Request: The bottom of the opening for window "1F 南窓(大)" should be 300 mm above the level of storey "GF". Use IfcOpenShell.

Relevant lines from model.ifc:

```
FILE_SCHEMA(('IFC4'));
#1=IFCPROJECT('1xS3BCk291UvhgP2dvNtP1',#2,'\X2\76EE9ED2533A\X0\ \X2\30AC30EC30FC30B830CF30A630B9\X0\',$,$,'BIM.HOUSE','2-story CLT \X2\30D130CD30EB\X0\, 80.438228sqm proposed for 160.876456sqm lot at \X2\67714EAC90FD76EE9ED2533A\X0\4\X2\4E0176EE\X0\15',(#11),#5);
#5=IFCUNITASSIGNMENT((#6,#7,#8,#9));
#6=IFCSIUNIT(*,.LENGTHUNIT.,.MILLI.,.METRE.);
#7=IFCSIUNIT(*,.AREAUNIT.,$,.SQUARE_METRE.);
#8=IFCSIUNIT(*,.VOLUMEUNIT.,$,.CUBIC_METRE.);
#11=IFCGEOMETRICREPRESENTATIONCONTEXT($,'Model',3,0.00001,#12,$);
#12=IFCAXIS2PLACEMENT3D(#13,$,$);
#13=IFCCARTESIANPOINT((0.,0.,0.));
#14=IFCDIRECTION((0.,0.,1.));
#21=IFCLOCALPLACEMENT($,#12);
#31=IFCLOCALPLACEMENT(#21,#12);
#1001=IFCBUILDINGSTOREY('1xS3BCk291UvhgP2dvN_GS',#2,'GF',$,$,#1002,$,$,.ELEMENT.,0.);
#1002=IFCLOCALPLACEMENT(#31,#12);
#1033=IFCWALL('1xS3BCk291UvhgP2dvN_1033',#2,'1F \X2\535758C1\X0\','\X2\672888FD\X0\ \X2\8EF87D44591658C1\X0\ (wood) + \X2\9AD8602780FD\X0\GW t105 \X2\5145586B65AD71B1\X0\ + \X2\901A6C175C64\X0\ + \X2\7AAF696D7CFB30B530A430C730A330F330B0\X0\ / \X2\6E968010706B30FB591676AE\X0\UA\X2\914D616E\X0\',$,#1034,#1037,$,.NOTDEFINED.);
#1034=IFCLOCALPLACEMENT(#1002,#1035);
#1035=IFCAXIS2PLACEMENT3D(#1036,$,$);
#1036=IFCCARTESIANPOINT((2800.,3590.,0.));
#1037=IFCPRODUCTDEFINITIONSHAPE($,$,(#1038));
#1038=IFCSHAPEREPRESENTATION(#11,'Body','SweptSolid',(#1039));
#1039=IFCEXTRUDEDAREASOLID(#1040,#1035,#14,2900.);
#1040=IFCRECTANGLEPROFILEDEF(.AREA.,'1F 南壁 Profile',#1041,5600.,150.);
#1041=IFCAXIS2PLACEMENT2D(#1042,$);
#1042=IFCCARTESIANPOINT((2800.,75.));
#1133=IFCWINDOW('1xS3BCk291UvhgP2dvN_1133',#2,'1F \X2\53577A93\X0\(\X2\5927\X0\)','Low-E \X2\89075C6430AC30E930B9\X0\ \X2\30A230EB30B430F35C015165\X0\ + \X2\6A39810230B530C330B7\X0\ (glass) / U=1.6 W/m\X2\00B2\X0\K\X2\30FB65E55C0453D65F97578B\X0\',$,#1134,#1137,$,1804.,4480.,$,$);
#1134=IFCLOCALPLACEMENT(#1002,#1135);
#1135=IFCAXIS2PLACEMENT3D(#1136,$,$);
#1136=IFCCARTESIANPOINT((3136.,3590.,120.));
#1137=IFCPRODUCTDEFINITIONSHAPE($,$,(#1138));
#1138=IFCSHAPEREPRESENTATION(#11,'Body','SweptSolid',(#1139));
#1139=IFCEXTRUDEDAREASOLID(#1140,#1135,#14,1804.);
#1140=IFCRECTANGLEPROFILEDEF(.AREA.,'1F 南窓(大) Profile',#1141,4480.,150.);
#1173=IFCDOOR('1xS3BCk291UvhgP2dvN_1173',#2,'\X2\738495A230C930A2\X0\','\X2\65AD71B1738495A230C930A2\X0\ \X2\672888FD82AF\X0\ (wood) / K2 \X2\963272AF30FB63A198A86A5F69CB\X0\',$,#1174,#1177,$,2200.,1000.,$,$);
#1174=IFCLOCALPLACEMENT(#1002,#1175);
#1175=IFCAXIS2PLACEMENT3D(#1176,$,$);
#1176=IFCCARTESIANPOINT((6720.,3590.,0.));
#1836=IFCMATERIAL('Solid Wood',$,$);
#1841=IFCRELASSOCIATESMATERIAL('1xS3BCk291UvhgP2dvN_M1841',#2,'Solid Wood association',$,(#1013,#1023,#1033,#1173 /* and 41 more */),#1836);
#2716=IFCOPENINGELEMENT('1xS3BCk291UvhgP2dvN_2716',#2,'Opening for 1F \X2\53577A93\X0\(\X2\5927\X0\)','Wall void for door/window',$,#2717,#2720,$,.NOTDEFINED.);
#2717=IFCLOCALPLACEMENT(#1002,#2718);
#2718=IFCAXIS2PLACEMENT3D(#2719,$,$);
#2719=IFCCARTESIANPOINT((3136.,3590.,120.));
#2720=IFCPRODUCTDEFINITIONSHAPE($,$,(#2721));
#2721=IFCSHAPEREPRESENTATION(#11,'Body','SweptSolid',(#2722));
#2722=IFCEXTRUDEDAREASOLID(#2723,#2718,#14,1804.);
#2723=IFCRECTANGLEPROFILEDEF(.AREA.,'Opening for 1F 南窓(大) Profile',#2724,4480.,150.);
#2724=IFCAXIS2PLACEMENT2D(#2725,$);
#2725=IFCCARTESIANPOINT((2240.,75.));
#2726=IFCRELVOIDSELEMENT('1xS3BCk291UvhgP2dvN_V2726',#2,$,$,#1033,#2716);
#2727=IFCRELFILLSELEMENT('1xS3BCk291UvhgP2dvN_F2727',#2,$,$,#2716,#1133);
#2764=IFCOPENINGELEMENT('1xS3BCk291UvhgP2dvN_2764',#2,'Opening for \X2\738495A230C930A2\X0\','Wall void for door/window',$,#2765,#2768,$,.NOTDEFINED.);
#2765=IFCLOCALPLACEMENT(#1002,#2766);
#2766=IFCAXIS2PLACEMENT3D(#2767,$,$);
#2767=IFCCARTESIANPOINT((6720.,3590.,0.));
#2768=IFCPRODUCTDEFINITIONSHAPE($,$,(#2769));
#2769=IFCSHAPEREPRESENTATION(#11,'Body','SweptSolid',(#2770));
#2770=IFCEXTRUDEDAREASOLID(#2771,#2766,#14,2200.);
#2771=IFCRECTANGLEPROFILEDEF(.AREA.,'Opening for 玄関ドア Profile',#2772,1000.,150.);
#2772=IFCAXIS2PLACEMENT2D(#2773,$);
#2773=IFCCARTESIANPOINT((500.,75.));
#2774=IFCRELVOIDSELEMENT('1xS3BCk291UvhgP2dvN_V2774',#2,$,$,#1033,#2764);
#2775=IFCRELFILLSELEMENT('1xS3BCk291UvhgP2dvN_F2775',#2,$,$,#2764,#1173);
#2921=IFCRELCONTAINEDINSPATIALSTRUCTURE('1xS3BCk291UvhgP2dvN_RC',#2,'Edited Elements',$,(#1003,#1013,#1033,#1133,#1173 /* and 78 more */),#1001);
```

```python
import numpy as np
import ifcopenshell
import ifcopenshell.api.geometry
import ifcopenshell.geom
import ifcopenshell.util.element
import ifcopenshell.util.placement
import ifcopenshell.util.shape
import ifcopenshell.util.unit

model = ifcopenshell.open("model.ifc")
unit_scale = ifcopenshell.util.unit.calculate_unit_scale(model)

window = model.by_guid("1xS3BCk291UvhgP2dvN_1133")
opening = window.FillsVoids[0].RelatingOpeningElement
storey = ifcopenshell.util.element.get_container(window, ifc_class="IfcBuildingStorey")
level = ifcopenshell.util.placement.get_local_placement(storey.ObjectPlacement)[2, 3]

# The opening's origin need not be at the sill, so measure its lowest point.
shape = ifcopenshell.geom.create_shape(ifcopenshell.geom.settings(), opening)
bottom = ifcopenshell.util.shape.get_shape_bottom_elevation(shape, shape.geometry) / unit_scale
dz = level + 0.3 / unit_scale - bottom

shift = np.array([0.0, 0.0, dz])
# The window is not placed relative to its opening, so move both.
for product in (opening, window):
    matrix = ifcopenshell.util.placement.get_local_placement(product.ObjectPlacement)
    matrix[:3, 3] += shift
    ifcopenshell.api.geometry.edit_object_placement(model, product=product, matrix=matrix, is_si=False)

print(f"moved by {dz * unit_scale:+.3f} m")

model.write("model_edited.ifc")
```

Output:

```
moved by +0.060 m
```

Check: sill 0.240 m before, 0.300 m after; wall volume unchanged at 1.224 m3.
